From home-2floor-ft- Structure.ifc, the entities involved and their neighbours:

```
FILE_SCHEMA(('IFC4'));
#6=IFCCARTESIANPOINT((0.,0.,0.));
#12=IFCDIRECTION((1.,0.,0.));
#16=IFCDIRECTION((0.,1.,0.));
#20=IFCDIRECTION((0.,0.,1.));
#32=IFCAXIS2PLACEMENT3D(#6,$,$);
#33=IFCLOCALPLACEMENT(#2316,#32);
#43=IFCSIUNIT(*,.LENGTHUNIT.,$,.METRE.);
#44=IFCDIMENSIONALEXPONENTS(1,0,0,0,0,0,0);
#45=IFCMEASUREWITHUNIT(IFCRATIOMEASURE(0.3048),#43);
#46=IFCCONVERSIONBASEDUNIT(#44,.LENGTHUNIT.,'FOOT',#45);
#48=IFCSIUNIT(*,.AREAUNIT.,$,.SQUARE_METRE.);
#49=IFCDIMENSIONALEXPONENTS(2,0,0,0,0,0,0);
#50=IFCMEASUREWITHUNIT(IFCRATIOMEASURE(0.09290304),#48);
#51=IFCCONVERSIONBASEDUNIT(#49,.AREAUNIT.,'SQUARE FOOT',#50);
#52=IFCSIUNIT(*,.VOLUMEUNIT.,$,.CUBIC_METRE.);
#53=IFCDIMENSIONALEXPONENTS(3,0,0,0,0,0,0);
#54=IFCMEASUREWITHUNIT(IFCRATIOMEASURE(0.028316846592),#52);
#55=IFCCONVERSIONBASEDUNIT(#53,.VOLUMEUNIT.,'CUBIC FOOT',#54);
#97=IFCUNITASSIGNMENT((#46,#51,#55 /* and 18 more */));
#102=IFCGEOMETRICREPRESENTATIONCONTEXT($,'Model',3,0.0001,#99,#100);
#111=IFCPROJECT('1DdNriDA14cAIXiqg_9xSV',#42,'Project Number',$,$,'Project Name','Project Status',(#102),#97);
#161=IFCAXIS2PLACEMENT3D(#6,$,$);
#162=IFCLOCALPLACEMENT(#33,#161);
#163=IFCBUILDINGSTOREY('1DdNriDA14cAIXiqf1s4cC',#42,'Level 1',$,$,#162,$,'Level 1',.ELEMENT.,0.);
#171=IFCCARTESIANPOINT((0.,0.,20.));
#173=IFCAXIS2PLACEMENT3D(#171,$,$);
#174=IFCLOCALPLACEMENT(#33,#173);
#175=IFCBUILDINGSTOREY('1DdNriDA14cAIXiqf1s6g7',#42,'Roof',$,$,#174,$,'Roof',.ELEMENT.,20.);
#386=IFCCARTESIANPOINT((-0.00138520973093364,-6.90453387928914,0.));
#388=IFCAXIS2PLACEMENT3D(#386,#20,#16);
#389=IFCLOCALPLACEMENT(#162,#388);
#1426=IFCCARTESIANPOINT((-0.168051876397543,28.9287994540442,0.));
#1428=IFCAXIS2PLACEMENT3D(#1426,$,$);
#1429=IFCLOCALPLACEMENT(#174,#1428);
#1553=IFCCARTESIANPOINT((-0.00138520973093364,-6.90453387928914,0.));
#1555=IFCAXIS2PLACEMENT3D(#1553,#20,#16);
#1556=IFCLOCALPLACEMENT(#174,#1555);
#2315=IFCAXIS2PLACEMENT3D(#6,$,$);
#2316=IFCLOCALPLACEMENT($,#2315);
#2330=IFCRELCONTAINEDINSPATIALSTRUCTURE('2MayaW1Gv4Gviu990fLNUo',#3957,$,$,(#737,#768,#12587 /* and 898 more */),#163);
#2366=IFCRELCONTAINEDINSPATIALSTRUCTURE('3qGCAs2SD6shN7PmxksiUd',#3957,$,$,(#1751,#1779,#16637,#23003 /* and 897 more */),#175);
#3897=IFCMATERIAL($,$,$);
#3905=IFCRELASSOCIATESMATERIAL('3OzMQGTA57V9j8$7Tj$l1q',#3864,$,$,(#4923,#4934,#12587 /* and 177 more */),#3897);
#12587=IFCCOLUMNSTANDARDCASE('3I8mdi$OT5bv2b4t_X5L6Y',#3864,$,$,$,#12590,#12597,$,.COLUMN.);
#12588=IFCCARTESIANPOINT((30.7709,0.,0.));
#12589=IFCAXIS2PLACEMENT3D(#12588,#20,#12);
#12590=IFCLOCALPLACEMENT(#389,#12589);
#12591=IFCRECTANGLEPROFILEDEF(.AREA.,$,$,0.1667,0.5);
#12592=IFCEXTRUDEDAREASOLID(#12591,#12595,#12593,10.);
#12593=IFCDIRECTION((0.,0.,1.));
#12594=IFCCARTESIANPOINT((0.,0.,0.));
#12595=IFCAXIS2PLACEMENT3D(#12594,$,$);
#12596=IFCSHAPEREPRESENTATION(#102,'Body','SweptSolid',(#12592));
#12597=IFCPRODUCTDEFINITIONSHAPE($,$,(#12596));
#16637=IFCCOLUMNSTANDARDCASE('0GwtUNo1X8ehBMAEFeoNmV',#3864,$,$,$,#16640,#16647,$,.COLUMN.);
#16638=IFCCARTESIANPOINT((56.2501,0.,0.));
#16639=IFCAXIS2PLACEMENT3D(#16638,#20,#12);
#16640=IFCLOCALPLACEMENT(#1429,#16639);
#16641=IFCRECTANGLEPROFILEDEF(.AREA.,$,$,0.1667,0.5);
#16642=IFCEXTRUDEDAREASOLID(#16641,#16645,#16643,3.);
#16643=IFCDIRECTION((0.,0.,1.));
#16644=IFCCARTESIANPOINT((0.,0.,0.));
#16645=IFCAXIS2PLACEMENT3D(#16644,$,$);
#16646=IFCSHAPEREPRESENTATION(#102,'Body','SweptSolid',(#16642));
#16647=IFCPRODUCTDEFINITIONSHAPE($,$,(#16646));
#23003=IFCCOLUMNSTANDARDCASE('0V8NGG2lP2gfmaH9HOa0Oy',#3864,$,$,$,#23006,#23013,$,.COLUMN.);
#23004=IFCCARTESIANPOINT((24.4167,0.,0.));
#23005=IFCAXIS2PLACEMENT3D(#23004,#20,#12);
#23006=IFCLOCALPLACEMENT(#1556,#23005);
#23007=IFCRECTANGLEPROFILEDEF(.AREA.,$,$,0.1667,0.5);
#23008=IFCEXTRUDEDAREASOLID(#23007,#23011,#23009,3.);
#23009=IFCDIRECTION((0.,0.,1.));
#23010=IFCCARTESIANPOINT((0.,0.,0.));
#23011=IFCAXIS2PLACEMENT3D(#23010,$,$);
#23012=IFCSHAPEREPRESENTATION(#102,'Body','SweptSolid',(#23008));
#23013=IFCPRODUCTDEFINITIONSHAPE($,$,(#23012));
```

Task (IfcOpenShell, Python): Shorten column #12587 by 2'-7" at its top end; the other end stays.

```python
import ifcopenshell
import ifcopenshell.util.unit

model = ifcopenshell.open("home-2floor-ft- Structure.ifc")
unit_scale = ifcopenshell.util.unit.calculate_unit_scale(model)

member = model.by_id(12587)
change = -31 * 0.0254 / unit_scale

# The extrusion runs towards the end named, so only its depth changes.
body = next(r for r in member.Representation.Representations if r.RepresentationIdentifier == "Body")
solid = body.Items[0]
old_length = solid.Depth
solid.Depth += change

print(f"length {old_length:g} -> {solid.Depth:g}")

model.write("home-2floor-ft- Structure_edited.ifc")
```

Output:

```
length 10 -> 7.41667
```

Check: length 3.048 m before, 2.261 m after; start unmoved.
